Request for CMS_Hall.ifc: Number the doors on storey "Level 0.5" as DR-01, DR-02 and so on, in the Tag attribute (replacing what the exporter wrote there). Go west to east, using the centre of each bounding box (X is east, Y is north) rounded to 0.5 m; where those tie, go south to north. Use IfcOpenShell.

First a look at what the model holds.

```python
import ifcopenshell
import ifcopenshell.util.element
import ifcopenshell.util.placement

model = ifcopenshell.open("CMS_Hall.ifc")
print(model.schema)
storey = next(s for s in model.by_type("IfcBuildingStorey") if s.Name == "Level 0.5")
doors = [e for e in ifcopenshell.util.element.get_decomposition(storey) if e.is_a("IfcDoor")]
for e in sorted(doors, key=lambda e: e.id()):
    origin = ifcopenshell.util.placement.get_local_placement(e.ObjectPlacement)[:3, 3]
    print(e.id(), e.Tag, e.Name, origin.round(2) + 0.0, sep=" | ")
```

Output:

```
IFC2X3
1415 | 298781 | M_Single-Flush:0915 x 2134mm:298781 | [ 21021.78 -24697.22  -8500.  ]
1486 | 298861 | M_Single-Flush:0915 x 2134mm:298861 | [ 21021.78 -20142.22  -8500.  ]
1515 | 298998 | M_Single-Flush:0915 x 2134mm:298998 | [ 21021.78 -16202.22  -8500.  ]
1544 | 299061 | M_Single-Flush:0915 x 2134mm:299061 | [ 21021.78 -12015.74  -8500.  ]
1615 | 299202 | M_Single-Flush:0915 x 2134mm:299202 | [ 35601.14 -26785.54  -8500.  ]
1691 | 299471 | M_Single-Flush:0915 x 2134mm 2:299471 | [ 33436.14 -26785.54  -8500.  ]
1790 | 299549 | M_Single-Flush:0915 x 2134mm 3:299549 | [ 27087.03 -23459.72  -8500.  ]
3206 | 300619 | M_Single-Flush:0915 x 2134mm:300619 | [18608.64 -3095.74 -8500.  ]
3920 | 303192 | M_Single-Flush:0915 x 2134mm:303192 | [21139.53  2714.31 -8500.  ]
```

```python
import ifcopenshell
import ifcopenshell.geom
import ifcopenshell.util.element
import ifcopenshell.util.shape

model = ifcopenshell.open("CMS_Hall.ifc")
settings = ifcopenshell.geom.settings()
settings.set("use-world-coords", True)


def centre(element):
    shape = ifcopenshell.geom.create_shape(settings, element)
    return ifcopenshell.util.shape.get_bbox_centroid(shape.geometry)


storey = next(s for s in model.by_type("IfcBuildingStorey") if s.Name == "Level 0.5")
doors = [e for e in ifcopenshell.util.element.get_decomposition(storey) if e.is_a("IfcDoor")]

# Insertion points can sit at a corner or the storey origin, so sort by the geometry (in metres).
centres = {e: centre(e) for e in doors}
doors.sort(key=lambda e: (round(centres[e][0] / 0.5), centres[e][1]))

for i, e in enumerate(doors, start=1):
    number = f"DR-{i:02d}"
    e.Tag = number
    print(e.id(), number)

model.write("CMS_Hall_edited.ifc")
```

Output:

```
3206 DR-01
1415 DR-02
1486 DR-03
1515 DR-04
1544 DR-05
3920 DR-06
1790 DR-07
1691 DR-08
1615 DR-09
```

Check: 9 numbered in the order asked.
